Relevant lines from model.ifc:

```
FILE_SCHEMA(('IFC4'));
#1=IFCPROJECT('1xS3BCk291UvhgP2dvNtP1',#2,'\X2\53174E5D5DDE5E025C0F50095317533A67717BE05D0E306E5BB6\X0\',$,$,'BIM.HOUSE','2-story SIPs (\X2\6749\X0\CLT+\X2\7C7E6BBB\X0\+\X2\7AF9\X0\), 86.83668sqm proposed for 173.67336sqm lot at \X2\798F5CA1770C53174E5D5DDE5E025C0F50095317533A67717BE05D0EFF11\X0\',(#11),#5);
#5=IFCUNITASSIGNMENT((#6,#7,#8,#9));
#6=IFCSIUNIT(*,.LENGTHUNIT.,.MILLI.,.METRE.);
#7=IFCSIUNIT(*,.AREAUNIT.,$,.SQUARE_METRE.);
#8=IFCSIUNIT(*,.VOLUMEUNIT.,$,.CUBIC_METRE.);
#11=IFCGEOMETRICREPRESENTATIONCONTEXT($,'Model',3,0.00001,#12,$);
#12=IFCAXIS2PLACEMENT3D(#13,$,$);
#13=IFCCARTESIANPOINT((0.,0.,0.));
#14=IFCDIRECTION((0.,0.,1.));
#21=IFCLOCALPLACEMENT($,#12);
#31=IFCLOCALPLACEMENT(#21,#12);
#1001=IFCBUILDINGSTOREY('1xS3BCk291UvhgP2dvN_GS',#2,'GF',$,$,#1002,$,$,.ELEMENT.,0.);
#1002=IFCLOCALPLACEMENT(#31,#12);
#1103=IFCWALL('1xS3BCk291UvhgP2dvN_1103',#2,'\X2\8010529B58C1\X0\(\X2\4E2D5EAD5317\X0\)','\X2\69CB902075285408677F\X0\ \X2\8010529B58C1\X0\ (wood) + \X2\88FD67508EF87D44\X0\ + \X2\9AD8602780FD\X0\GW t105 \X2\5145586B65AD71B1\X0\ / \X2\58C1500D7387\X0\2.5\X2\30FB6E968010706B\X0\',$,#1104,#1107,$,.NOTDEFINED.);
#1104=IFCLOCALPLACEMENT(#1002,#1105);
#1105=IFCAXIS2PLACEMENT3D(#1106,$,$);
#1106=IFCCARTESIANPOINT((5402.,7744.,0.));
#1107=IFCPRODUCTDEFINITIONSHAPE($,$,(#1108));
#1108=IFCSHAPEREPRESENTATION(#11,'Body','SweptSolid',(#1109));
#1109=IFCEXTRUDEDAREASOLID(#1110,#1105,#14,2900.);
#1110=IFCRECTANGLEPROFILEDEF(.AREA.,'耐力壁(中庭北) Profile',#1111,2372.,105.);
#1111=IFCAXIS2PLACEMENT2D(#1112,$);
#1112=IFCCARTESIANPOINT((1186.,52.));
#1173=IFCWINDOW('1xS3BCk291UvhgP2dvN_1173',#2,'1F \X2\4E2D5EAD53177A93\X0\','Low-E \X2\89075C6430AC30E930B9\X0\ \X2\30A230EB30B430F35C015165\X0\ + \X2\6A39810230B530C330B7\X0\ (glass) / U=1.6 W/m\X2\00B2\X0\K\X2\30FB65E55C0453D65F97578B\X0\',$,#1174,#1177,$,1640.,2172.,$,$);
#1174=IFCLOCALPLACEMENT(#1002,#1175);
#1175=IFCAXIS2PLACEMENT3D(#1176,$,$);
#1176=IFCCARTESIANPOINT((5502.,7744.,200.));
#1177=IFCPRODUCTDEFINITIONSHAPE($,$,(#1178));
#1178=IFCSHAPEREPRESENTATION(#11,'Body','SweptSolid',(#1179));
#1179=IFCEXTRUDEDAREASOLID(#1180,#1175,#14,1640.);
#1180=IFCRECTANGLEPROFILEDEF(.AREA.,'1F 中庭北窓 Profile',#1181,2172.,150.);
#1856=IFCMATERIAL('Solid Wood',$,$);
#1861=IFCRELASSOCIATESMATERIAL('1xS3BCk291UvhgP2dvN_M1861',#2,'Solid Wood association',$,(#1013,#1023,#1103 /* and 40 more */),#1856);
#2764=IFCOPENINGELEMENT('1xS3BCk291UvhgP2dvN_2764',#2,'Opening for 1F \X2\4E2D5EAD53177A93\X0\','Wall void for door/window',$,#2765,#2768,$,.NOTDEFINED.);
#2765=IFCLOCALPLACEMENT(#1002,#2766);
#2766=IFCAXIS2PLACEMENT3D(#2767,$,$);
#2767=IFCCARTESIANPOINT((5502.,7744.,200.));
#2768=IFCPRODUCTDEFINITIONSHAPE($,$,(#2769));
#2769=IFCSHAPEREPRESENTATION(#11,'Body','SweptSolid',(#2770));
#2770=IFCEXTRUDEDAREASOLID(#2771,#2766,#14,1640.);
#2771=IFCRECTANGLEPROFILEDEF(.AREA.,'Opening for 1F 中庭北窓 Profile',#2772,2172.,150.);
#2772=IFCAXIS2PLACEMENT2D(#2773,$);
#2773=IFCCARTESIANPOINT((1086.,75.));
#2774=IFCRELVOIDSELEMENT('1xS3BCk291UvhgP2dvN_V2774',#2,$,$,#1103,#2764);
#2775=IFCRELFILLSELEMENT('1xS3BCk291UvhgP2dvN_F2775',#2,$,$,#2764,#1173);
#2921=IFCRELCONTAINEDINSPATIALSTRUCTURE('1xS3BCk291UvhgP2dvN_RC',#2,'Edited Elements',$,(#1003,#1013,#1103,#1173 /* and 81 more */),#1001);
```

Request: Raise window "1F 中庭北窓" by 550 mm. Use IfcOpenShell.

```python
import numpy as np
import ifcopenshell
import ifcopenshell.api.geometry
import ifcopenshell.util.placement
import ifcopenshell.util.unit

model = ifcopenshell.open("model.ifc")
unit_scale = ifcopenshell.util.unit.calculate_unit_scale(model)

window = model.by_id(1173)
opening = window.FillsVoids[0].RelatingOpeningElement
dz = 0.55 / unit_scale

shift = np.array([0.0, 0.0, dz])
# The window is not placed relative to its opening, so move both.
for product in (opening, window):
    matrix = ifcopenshell.util.placement.get_local_placement(product.ObjectPlacement)
    matrix[:3, 3] += shift
    ifcopenshell.api.geometry.edit_object_placement(model, product=product, matrix=matrix, is_si=False)

print(f"moved by {dz * unit_scale:+.3f} m")

model.write("model_rev.ifc")
```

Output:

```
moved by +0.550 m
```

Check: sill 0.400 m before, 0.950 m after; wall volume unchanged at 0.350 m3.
